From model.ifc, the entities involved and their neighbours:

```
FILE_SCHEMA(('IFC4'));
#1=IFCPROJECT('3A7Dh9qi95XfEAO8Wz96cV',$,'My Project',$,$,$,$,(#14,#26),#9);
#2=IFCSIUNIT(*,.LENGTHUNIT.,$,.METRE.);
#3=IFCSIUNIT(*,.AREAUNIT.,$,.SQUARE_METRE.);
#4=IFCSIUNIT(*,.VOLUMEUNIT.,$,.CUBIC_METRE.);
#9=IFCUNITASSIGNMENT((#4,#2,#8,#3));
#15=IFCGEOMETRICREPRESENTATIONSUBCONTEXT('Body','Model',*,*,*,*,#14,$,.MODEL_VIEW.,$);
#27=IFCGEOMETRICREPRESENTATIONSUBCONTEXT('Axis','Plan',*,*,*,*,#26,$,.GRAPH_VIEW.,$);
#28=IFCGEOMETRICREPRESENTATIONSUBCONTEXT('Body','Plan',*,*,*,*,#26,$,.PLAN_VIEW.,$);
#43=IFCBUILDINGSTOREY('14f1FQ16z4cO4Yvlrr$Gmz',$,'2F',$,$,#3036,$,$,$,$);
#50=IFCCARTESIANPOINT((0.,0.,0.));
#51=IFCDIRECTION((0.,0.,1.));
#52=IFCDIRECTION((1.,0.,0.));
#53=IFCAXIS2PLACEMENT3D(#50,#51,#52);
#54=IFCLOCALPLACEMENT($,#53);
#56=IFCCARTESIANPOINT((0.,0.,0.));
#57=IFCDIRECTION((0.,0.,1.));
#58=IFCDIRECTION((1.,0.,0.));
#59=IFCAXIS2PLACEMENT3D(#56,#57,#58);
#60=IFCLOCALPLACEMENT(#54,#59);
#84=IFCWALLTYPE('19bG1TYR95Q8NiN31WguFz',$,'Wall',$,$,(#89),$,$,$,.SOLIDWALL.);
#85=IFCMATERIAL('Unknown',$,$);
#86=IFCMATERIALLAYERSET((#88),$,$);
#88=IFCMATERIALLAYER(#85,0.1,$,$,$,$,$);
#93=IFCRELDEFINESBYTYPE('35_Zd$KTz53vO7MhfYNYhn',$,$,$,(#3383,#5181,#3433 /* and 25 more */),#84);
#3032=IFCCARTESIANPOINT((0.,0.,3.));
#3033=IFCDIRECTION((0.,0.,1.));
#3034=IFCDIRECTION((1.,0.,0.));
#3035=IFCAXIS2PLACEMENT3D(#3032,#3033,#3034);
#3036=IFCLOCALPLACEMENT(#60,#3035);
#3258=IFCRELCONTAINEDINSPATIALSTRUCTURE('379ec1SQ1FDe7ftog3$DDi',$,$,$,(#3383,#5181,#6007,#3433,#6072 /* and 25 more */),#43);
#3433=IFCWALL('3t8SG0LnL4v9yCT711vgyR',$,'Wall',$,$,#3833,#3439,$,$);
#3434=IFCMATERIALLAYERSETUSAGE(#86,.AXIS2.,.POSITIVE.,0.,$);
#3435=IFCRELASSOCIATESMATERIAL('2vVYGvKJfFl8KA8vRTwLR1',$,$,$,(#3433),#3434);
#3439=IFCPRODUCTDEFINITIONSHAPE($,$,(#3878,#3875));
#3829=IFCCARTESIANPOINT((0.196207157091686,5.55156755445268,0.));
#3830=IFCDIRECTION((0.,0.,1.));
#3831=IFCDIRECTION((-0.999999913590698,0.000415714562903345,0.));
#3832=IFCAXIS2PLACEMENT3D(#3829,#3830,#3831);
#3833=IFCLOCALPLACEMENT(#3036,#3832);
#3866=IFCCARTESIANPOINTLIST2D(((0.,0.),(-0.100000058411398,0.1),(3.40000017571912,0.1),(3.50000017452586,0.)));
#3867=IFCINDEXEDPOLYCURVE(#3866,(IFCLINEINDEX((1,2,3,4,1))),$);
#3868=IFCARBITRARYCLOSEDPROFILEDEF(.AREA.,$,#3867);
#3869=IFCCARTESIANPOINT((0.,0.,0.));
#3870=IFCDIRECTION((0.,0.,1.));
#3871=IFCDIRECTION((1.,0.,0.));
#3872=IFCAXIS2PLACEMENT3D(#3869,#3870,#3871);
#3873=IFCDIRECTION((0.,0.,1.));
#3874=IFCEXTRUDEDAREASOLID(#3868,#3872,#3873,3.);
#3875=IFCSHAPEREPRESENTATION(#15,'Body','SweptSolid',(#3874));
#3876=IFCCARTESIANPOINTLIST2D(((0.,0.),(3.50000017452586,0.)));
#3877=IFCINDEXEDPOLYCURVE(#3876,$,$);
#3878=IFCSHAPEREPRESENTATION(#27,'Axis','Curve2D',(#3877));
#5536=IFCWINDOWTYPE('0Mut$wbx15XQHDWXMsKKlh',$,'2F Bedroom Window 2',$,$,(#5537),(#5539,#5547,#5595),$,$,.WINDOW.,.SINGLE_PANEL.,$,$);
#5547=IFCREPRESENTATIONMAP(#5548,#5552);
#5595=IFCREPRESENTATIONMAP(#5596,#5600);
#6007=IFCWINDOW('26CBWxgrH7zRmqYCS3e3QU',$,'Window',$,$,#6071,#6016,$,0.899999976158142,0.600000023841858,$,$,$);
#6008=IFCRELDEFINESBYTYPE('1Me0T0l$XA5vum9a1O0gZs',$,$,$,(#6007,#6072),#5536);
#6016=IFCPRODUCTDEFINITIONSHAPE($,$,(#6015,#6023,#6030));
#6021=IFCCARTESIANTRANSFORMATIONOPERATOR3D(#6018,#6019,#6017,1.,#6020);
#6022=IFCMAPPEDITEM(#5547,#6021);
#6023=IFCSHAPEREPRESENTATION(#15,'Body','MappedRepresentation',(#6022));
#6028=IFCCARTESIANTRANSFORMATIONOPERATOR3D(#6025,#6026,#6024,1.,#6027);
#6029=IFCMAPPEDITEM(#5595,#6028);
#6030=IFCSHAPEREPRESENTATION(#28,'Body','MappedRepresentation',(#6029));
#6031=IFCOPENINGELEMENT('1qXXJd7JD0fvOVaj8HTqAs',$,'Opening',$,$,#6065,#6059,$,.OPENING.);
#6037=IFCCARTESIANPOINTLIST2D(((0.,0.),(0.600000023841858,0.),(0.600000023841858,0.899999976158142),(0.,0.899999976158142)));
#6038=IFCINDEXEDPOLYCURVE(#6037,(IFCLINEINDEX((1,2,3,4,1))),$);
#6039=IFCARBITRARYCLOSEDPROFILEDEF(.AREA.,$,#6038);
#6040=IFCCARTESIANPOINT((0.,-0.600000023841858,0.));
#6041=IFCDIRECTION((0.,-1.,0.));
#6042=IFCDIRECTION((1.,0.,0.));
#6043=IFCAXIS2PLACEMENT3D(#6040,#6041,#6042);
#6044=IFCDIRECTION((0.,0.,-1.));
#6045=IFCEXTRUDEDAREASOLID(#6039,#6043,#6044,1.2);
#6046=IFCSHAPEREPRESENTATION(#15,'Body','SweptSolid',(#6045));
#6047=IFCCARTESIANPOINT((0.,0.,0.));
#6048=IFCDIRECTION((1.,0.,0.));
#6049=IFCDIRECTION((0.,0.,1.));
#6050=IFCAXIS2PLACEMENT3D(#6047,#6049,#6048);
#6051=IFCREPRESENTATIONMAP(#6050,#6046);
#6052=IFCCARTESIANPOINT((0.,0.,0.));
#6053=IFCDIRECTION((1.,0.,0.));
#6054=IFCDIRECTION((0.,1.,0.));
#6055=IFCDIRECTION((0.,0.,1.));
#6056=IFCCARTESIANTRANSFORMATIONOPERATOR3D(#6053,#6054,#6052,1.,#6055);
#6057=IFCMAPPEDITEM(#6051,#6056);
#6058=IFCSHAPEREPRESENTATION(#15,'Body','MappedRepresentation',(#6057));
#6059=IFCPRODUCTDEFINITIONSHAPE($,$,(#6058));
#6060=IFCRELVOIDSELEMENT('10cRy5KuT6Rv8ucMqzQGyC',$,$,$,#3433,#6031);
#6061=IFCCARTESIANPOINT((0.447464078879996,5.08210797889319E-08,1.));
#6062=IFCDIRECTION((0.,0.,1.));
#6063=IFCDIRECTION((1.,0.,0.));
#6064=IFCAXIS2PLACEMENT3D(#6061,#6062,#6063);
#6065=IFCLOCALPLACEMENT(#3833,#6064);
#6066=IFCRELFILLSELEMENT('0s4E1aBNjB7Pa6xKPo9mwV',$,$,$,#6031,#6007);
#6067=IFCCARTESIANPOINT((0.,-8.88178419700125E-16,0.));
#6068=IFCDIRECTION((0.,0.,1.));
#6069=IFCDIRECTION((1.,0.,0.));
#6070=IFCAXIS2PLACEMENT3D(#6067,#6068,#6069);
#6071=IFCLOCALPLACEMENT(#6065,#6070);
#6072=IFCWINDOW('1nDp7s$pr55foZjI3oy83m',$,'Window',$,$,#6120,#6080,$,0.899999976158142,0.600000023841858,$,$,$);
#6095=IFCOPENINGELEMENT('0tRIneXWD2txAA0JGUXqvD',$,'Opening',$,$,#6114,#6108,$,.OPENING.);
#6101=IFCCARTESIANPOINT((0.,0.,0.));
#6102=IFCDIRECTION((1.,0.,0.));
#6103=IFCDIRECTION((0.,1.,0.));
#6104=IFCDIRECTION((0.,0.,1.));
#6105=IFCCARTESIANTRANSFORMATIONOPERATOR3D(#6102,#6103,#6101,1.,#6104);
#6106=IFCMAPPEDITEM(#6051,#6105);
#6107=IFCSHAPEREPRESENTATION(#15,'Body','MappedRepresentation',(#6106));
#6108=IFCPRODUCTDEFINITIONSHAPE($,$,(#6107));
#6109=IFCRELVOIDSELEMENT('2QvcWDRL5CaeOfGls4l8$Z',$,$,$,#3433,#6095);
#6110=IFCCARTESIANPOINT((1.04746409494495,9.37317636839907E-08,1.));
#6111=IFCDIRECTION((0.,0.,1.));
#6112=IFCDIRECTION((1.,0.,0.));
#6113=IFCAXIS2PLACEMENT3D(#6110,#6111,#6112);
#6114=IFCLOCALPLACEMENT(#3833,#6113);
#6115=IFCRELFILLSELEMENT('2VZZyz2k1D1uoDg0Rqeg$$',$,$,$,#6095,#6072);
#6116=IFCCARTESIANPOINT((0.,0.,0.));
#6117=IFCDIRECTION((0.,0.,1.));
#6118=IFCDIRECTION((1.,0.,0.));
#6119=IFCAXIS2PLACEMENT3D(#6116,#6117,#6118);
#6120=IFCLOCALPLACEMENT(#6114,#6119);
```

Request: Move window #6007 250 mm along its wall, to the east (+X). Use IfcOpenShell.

```python
import ifcopenshell
import ifcopenshell.api.geometry
import ifcopenshell.util.placement
import ifcopenshell.util.unit

model = ifcopenshell.open("model.ifc")
unit_scale = ifcopenshell.util.unit.calculate_unit_scale(model)

window = model.by_id(6007)
opening = window.FillsVoids[0].RelatingOpeningElement
wall = opening.VoidsElements[0].RelatingBuildingElement

wall_matrix = ifcopenshell.util.placement.get_local_placement(wall.ObjectPlacement)
shift = wall_matrix[:3, 0] * -0.25 / unit_scale
before = ifcopenshell.util.placement.get_local_placement(window.ObjectPlacement)[:3, 3].copy()

# The window is placed relative to its opening, so it follows when the opening moves.
matrix = ifcopenshell.util.placement.get_local_placement(opening.ObjectPlacement)
matrix[:3, 3] += shift
ifcopenshell.api.geometry.edit_object_placement(
    model, product=opening, matrix=matrix, is_si=False, should_transform_children=True
)

after = ifcopenshell.util.placement.get_local_placement(window.ObjectPlacement)[:3, 3]
print("window moved by", (after - before).round(3) + 0.0)

model.write("model-out.ifc")
```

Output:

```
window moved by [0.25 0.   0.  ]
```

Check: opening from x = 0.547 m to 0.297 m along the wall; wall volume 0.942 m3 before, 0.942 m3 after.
